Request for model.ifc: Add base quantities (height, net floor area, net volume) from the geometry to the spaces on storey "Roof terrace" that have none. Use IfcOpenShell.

First a look at what the model holds.

```python
import ifcopenshell
import ifcopenshell.util.element
import ifcopenshell.util.unit

model = ifcopenshell.open("model.ifc")
print(model.schema)
for unit_type in ("LENGTHUNIT", "AREAUNIT", "VOLUMEUNIT"):
    print(unit_type, ifcopenshell.util.unit.calculate_unit_scale(model, unit_type))
storey = next(s for s in model.by_type("IfcBuildingStorey") if s.Name == "Roof terrace")
spaces = [e for e in ifcopenshell.util.element.get_decomposition(storey) if e.is_a("IfcSpace")]
for e in sorted(spaces, key=lambda e: e.id()):
    print(e.id(), e.is_a(), e.Name, list(ifcopenshell.util.element.get_psets(e, qtos_only=True)), sep=" | ")
```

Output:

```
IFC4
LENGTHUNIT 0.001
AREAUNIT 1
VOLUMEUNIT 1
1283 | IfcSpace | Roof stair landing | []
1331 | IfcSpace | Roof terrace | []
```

```python
import ifcopenshell
import ifcopenshell.api.pset
import ifcopenshell.geom
import ifcopenshell.util.element
import ifcopenshell.util.shape
import ifcopenshell.util.unit

model = ifcopenshell.open("model.ifc")
unit_scale = ifcopenshell.util.unit.calculate_unit_scale(model)
area_scale = ifcopenshell.util.unit.calculate_unit_scale(model, "AREAUNIT")
volume_scale = ifcopenshell.util.unit.calculate_unit_scale(model, "VOLUMEUNIT")
settings = ifcopenshell.geom.settings()

storey = next(s for s in model.by_type("IfcBuildingStorey") if s.Name == "Roof terrace")
spaces = [e for e in ifcopenshell.util.element.get_decomposition(storey) if e.is_a("IfcSpace")]

for e in sorted(spaces, key=lambda e: e.id()):
    if ifcopenshell.util.element.get_psets(e, qtos_only=True, should_inherit=False):
        continue
    # Geometry comes back in metres, in the element's own axes.
    shape = ifcopenshell.geom.create_shape(settings, e)
    values = {
        "Height": ifcopenshell.util.shape.get_z(shape.geometry) / unit_scale,
        "NetFloorArea": ifcopenshell.util.shape.get_footprint_area(shape.geometry) / area_scale,
        "NetVolume": ifcopenshell.util.shape.get_volume(shape.geometry) / volume_scale,
    }
    qto = ifcopenshell.api.pset.add_qto(model, product=e, name="Qto_SpaceBaseQuantities")
    ifcopenshell.api.pset.edit_qto(model, qto=qto, properties=values)
    print(e.id(), {k: round(v, 3) for k, v in values.items()})

model.write("model_updated.ifc")
```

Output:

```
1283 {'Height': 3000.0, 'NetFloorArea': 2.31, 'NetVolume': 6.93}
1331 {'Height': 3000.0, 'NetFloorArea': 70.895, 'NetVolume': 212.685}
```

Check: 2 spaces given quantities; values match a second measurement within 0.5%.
